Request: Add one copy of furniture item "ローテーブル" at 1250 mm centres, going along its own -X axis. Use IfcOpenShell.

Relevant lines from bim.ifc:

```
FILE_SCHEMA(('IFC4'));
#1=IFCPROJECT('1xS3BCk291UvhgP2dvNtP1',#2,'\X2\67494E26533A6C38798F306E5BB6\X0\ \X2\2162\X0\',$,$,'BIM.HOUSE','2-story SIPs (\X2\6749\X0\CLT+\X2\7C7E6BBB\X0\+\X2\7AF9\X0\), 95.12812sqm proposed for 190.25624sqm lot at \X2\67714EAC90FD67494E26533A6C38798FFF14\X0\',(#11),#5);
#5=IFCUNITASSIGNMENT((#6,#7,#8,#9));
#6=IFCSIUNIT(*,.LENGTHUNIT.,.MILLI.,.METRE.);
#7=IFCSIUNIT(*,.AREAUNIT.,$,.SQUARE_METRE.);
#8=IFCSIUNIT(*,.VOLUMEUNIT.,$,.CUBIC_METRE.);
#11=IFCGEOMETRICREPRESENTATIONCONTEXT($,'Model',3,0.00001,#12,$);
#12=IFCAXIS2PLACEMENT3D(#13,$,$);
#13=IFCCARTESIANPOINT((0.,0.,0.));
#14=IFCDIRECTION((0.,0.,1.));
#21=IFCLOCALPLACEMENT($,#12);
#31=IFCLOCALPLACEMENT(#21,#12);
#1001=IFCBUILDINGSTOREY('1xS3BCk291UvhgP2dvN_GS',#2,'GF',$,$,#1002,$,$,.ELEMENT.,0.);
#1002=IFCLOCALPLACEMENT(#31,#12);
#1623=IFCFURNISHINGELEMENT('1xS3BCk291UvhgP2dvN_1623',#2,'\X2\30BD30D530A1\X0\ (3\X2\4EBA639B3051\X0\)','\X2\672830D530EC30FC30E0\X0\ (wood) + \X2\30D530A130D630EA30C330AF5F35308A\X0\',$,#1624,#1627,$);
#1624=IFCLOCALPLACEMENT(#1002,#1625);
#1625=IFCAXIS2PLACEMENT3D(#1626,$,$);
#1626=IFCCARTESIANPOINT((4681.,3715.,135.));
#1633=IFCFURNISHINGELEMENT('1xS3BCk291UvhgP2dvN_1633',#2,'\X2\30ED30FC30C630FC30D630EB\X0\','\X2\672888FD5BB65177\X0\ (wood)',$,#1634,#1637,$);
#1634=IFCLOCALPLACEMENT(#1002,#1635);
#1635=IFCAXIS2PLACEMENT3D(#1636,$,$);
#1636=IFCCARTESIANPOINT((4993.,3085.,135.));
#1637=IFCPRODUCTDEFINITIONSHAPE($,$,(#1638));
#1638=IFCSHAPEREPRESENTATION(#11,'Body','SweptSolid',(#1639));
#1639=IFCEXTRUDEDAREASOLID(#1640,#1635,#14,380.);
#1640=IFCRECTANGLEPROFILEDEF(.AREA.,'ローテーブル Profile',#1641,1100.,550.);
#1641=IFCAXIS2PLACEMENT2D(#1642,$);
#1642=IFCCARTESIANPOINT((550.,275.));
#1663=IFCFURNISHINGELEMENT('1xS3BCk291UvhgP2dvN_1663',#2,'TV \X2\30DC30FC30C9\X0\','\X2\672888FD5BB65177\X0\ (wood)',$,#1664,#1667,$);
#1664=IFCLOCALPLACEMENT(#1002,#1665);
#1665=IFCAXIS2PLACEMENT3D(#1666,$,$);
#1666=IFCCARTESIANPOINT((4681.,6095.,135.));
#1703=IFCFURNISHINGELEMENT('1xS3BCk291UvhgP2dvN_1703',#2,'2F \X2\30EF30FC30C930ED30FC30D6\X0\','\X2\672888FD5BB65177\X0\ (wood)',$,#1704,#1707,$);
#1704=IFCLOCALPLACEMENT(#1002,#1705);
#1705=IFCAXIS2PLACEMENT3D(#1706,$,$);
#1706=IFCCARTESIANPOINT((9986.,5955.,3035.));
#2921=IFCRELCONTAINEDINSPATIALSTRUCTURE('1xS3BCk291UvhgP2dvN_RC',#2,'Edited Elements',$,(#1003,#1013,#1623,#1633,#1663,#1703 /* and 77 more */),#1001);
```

```python
import ifcopenshell
import ifcopenshell.api.geometry
import ifcopenshell.api.root
import ifcopenshell.util.element
import ifcopenshell.util.placement

model = ifcopenshell.open("bim.ifc")


def reuse_history(source, copy):
    """copy_class also copies each property set's owner history, people and application; keep the originals."""
    for rel in copy.IsDefinedBy:
        if rel.is_a("IfcRelDefinesByProperties") and (history := rel.RelatingPropertyDefinition.OwnerHistory):
            rel.RelatingPropertyDefinition.OwnerHistory = source.OwnerHistory
            ifcopenshell.util.element.remove_deep2(model, history)


source = model.by_guid("1xS3BCk291UvhgP2dvN_1633")
base = ifcopenshell.util.placement.get_local_placement(source.ObjectPlacement)
step = -base[:3, 0] * 1250.0

for i in range(1, 2):
    copy = ifcopenshell.api.root.copy_class(model, product=source)
    copy.Representation = ifcopenshell.util.element.copy_deep(
        model, source.Representation, exclude=["IfcGeometricRepresentationContext", "IfcRepresentationMap"]
    )
    reuse_history(source, copy)
    matrix = base.copy()
    matrix[:3, 3] += i * step
    print("added at", matrix[:3, 3].round(3) + 0.0)
    ifcopenshell.api.geometry.edit_object_placement(model, product=copy, matrix=matrix, is_si=False)

model.write("bim_updated.ifc")
```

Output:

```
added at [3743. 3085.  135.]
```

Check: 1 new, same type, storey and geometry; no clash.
